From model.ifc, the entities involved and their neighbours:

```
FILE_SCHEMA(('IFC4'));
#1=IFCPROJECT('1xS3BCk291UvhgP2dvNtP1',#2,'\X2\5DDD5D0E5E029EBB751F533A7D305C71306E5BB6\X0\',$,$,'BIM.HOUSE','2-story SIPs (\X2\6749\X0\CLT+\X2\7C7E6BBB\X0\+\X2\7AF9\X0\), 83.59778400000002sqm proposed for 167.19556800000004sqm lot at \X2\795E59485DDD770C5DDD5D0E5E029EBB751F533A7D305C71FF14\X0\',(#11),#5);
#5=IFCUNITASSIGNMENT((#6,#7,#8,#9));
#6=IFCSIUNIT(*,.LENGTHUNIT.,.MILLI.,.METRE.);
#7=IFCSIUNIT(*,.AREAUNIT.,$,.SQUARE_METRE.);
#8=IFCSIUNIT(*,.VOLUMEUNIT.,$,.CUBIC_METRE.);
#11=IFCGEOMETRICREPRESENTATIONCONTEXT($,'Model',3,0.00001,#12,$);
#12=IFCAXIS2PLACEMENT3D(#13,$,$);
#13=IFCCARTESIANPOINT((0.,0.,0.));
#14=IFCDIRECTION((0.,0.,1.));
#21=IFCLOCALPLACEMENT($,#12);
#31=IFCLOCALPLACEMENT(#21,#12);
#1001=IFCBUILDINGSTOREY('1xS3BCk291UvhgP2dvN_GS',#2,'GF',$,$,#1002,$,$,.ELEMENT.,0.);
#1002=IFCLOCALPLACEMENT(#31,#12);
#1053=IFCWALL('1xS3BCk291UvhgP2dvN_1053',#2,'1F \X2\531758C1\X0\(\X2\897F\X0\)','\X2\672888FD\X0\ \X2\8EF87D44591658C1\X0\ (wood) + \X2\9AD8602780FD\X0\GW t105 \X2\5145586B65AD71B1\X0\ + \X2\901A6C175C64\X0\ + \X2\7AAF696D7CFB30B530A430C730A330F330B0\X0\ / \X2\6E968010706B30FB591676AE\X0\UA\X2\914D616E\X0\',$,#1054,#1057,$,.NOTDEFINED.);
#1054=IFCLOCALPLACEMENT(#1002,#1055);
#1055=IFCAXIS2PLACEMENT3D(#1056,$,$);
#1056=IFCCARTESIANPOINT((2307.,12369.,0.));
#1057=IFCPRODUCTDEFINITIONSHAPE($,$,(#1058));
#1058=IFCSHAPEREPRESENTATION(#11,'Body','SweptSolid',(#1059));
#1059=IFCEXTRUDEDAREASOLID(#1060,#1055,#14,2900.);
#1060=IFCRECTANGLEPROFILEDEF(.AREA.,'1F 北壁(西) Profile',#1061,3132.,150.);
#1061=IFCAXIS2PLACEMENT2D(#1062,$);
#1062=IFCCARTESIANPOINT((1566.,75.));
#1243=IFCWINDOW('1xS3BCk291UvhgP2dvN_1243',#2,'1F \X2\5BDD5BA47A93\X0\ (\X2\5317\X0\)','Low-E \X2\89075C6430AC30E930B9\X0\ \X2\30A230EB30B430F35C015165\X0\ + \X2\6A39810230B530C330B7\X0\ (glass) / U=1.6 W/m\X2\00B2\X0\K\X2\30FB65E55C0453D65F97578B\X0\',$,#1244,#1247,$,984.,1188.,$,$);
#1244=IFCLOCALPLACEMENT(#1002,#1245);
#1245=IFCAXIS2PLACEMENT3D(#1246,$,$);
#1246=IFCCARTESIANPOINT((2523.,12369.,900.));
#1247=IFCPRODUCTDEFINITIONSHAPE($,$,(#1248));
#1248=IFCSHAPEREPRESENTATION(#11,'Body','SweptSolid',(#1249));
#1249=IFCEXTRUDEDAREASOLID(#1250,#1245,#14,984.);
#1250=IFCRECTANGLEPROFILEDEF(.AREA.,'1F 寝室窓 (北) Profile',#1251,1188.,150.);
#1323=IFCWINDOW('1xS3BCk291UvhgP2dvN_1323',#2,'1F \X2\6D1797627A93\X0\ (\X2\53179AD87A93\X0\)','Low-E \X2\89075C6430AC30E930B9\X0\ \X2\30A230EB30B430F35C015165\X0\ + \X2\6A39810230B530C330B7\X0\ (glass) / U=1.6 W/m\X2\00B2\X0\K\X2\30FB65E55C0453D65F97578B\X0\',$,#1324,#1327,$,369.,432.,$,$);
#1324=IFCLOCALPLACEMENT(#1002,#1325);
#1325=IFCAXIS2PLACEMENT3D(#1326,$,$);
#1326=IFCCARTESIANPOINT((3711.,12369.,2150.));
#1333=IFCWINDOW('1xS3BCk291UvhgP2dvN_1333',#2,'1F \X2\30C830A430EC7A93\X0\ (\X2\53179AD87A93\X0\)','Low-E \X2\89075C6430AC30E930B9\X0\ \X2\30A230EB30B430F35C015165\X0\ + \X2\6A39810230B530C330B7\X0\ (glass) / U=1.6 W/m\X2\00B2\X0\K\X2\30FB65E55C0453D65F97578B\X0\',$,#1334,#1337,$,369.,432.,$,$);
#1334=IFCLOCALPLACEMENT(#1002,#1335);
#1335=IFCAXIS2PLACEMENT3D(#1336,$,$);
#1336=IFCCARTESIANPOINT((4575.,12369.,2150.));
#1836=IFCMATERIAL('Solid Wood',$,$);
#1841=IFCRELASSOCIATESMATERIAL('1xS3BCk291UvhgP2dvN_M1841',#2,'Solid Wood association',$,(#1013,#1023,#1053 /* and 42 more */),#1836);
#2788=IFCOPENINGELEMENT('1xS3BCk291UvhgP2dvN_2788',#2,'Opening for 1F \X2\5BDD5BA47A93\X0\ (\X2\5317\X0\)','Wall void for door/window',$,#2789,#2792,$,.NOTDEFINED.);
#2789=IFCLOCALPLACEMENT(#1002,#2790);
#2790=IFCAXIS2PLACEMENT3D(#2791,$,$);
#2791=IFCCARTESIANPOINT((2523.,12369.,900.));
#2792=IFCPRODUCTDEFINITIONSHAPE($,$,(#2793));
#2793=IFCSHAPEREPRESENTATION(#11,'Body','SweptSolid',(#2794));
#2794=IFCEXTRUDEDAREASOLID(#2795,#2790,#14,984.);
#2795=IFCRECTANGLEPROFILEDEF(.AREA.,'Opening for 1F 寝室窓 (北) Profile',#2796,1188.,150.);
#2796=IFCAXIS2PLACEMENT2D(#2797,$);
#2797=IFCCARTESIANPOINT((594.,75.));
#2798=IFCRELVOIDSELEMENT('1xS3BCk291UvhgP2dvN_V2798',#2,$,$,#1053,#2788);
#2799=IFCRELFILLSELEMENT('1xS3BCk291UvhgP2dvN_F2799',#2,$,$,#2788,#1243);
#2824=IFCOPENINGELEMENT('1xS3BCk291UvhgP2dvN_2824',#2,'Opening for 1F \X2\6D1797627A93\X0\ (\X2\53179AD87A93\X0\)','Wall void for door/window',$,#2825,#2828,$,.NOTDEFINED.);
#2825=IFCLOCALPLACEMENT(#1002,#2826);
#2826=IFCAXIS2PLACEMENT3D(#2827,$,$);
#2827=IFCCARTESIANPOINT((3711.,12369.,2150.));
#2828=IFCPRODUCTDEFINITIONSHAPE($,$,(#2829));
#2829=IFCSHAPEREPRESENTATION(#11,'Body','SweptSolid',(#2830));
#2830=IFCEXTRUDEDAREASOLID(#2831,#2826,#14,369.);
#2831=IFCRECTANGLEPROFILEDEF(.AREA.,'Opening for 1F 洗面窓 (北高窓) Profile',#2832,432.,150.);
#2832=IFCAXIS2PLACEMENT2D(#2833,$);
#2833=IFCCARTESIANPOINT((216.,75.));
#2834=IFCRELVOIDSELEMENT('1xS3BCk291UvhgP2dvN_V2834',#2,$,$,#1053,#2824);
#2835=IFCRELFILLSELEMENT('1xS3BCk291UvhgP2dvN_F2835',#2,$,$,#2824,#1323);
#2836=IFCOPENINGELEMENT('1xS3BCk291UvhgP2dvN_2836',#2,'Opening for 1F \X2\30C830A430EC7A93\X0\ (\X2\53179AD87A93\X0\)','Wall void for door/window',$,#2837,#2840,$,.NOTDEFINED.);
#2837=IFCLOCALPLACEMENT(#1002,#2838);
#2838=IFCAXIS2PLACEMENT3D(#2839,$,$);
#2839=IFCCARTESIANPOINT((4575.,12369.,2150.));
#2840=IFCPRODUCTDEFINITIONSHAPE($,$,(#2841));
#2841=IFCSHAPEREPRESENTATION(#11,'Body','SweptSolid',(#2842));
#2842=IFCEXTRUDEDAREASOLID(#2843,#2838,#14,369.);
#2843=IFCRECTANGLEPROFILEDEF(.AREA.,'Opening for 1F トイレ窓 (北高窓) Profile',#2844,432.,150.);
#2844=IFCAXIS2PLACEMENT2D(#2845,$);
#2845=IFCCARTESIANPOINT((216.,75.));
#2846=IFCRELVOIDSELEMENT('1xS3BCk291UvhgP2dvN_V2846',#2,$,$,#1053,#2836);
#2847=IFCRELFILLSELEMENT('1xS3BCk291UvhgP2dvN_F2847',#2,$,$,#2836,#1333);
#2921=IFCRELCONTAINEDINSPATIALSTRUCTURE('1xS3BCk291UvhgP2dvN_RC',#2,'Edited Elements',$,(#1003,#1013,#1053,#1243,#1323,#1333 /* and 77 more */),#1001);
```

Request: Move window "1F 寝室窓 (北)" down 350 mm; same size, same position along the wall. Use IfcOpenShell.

```python
import numpy as np
import ifcopenshell
import ifcopenshell.api.geometry
import ifcopenshell.util.placement
import ifcopenshell.util.unit

model = ifcopenshell.open("model.ifc")
unit_scale = ifcopenshell.util.unit.calculate_unit_scale(model)

window = model.by_guid("1xS3BCk291UvhgP2dvN_1243")
opening = window.FillsVoids[0].RelatingOpeningElement
dz = -0.35 / unit_scale

shift = np.array([0.0, 0.0, dz])
# The window is not placed relative to its opening, so move both.
for product in (opening, window):
    matrix = ifcopenshell.util.placement.get_local_placement(product.ObjectPlacement)
    matrix[:3, 3] += shift
    ifcopenshell.api.geometry.edit_object_placement(model, product=product, matrix=matrix, is_si=False)

print(f"moved by {dz * unit_scale:+.3f} m")

model.write("model-out.ifc")
```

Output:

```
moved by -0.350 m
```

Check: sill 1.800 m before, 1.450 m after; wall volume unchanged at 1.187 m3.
